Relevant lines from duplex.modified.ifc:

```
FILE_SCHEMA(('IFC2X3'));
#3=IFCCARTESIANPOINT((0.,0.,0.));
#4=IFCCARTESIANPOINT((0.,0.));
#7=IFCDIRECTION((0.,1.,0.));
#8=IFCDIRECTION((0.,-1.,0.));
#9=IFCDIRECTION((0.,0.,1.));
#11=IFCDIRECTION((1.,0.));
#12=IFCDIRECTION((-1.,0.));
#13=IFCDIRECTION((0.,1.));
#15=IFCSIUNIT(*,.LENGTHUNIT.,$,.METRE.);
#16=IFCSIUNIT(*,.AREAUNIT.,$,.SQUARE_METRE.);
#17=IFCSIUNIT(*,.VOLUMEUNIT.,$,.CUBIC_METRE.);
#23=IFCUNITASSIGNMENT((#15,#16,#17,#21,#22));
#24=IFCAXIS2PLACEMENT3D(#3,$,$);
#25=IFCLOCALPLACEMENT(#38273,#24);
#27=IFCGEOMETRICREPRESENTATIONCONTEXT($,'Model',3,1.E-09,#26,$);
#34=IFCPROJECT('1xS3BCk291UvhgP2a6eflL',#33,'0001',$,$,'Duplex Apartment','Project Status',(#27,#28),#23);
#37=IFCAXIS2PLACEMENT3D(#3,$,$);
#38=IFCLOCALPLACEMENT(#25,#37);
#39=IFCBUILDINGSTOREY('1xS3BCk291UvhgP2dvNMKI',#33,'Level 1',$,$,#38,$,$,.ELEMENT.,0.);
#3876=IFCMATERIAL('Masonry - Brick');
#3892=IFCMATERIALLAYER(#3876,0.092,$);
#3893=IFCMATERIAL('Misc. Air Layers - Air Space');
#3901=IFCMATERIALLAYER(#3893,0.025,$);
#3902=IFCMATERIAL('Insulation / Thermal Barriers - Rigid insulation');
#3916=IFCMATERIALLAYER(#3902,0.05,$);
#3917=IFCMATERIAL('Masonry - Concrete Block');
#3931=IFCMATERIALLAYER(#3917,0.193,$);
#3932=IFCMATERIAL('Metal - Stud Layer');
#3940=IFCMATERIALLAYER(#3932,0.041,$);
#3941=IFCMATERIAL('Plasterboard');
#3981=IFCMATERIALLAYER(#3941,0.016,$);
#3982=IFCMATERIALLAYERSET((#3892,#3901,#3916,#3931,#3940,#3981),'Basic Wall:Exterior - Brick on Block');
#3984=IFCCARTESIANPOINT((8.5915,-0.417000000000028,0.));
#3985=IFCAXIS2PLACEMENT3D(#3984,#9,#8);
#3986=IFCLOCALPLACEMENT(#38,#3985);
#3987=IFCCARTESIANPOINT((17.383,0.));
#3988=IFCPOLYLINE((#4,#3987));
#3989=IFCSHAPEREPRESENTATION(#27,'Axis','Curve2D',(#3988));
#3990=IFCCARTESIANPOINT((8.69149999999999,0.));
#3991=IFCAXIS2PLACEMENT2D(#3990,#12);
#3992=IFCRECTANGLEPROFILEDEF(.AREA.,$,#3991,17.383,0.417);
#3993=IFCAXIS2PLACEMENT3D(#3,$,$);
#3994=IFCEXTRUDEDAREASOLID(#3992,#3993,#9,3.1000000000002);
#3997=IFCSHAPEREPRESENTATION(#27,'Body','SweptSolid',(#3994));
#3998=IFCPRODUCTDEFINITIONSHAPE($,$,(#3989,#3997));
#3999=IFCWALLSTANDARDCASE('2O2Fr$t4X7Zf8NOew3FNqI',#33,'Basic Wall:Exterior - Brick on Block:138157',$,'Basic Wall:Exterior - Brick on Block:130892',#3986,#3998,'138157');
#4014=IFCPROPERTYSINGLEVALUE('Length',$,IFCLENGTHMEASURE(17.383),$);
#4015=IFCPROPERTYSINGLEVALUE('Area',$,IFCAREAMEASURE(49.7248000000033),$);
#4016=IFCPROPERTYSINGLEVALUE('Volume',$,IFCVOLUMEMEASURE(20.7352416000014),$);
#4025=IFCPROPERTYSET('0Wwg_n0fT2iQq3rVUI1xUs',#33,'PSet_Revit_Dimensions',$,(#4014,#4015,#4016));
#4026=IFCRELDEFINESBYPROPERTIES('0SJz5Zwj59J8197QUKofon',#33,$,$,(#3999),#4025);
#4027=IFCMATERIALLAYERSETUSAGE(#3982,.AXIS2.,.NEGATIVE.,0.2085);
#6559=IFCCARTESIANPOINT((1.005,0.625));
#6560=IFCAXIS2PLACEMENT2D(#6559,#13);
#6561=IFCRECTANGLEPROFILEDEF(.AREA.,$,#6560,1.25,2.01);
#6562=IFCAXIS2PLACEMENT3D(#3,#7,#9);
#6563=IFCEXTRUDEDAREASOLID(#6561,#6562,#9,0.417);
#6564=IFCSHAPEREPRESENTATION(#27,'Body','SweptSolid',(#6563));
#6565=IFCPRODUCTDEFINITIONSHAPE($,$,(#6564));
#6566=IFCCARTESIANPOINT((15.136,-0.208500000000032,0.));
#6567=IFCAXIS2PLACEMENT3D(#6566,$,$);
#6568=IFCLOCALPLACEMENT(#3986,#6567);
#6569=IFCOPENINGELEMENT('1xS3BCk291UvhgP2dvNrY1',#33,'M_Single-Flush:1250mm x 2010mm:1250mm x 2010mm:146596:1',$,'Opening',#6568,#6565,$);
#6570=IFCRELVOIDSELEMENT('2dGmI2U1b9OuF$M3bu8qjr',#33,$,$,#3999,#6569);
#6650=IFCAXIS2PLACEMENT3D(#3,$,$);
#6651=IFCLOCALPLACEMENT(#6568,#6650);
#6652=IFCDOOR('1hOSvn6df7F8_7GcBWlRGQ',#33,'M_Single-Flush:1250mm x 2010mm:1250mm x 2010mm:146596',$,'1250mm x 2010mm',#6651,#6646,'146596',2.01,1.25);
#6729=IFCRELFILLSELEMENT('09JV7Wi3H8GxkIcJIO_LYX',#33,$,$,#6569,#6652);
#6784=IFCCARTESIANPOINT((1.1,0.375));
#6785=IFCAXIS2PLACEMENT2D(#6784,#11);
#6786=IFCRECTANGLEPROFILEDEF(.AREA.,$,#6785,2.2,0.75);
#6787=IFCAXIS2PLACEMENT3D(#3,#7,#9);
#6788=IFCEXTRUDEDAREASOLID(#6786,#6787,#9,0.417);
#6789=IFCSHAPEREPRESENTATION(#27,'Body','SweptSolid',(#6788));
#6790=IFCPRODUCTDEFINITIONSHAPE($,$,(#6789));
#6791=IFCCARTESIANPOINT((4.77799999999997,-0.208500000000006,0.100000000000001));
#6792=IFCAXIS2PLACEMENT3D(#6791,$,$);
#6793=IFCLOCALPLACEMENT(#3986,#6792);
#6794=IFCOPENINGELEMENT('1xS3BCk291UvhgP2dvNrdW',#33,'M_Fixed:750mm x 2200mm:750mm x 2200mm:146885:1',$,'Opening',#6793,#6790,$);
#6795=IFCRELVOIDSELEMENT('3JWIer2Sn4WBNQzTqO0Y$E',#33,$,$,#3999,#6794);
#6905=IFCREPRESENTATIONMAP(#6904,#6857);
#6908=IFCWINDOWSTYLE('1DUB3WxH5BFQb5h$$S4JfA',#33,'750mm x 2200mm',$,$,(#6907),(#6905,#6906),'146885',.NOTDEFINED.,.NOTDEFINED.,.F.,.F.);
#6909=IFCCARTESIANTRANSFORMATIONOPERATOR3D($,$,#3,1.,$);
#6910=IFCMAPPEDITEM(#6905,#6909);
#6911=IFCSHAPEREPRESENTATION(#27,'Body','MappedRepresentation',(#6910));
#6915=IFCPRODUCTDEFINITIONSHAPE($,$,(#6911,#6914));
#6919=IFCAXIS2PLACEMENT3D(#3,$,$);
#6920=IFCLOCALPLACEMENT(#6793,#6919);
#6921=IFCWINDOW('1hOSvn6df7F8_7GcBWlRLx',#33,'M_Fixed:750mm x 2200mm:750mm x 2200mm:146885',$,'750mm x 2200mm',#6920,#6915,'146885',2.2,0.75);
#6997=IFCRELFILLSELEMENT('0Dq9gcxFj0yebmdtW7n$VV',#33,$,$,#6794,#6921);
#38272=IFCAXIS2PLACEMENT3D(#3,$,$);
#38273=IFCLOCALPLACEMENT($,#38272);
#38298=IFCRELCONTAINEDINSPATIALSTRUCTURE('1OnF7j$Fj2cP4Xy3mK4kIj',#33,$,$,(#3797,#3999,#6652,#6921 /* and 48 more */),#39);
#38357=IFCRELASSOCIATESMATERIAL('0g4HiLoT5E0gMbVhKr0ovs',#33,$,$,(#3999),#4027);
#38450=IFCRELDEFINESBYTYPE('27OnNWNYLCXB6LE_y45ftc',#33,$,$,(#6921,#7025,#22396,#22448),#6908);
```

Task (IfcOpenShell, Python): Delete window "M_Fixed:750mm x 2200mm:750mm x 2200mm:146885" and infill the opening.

```python
import ifcopenshell
import ifcopenshell.api.feature
import ifcopenshell.api.pset
import ifcopenshell.api.root
import ifcopenshell.geom
import ifcopenshell.util.element
import ifcopenshell.util.shape
import ifcopenshell.util.unit

model = ifcopenshell.open("duplex.modified.ifc")
area_scale = ifcopenshell.util.unit.calculate_unit_scale(model, "AREAUNIT")
volume_scale = ifcopenshell.util.unit.calculate_unit_scale(model, "VOLUMEUNIT")
settings = ifcopenshell.geom.settings()


def volume(element):
    """Net volume in cubic metres, openings subtracted."""
    shape = ifcopenshell.geom.create_shape(settings, element)
    return ifcopenshell.util.shape.get_volume(shape.geometry)


window = model.by_guid("1hOSvn6df7F8_7GcBWlRLx")
opening = window.FillsVoids[0].RelatingOpeningElement
wall = opening.VoidsElements[0].RelatingBuildingElement
before = volume(wall)

ifcopenshell.api.root.remove_product(model, product=window)
ifcopenshell.api.feature.remove_feature(model, feature=opening)

after = volume(wall)
thickness = 0.417  # wall thickness in metres

# Update the wall's stored quantities.
pset = model.by_id(ifcopenshell.util.element.get_pset(wall, "PSet_Revit_Dimensions", should_inherit=False)["id"])
ifcopenshell.api.pset.edit_pset(model, pset=pset, properties={
    "Area": model.create_entity("IfcAreaMeasure", after / thickness / area_scale),
    "Volume": model.create_entity("IfcVolumeMeasure", after / volume_scale),
})

print(f"wall volume {before:.3f} -> {after:.3f} m3")

model.write("duplex.modified_edited.ifc")
```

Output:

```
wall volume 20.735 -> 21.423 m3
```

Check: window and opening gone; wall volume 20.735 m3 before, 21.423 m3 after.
